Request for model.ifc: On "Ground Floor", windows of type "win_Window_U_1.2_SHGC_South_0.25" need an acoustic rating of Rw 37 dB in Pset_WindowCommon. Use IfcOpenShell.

First a look at what the model holds.

```python
import ifcopenshell
import ifcopenshell.util.element

model = ifcopenshell.open("model.ifc")
print(model.schema)
storey = next(s for s in model.by_type("IfcBuildingStorey") if s.Name == "Ground Floor")
windows = [e for e in ifcopenshell.util.element.get_decomposition(storey) if e.is_a("IfcWindow")]
seen = {}
for e in windows:
    element_type = ifcopenshell.util.element.get_type(e)
    key = (element_type.Name if element_type != e and element_type else None, ifcopenshell.util.element.get_pset(e, "Pset_WindowCommon", "AcousticRating"))
    seen[key] = seen.get(key, 0) + 1
for (name, value), count in sorted(seen.items(), key=str):
    print(count, "x", name, "|", value)
```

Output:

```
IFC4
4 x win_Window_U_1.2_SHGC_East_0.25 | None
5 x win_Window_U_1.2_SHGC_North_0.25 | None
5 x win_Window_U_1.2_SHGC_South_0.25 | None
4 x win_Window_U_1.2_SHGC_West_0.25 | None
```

```python
import ifcopenshell
import ifcopenshell.api.pset
import ifcopenshell.util.element

model = ifcopenshell.open("model.ifc")

storey = next(s for s in model.by_type("IfcBuildingStorey") if s.Name == "Ground Floor")
windows = [e for e in ifcopenshell.util.element.get_decomposition(storey) if e.is_a("IfcWindow")]

count = 0
for e in windows:
    element_type = ifcopenshell.util.element.get_type(e)
    if element_type in (None, e) or element_type.Name != "win_Window_U_1.2_SHGC_South_0.25":
        continue
    # add_pset returns the element's existing set when there is one.
    pset = ifcopenshell.api.pset.add_pset(model, product=e, name="Pset_WindowCommon")
    ifcopenshell.api.pset.edit_pset(model, pset=pset, properties={"AcousticRating": "Rw 37 dB"})
    count += 1

print(count, "windows updated")

model.write("model_v2.ifc")
```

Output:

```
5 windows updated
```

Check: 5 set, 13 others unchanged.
